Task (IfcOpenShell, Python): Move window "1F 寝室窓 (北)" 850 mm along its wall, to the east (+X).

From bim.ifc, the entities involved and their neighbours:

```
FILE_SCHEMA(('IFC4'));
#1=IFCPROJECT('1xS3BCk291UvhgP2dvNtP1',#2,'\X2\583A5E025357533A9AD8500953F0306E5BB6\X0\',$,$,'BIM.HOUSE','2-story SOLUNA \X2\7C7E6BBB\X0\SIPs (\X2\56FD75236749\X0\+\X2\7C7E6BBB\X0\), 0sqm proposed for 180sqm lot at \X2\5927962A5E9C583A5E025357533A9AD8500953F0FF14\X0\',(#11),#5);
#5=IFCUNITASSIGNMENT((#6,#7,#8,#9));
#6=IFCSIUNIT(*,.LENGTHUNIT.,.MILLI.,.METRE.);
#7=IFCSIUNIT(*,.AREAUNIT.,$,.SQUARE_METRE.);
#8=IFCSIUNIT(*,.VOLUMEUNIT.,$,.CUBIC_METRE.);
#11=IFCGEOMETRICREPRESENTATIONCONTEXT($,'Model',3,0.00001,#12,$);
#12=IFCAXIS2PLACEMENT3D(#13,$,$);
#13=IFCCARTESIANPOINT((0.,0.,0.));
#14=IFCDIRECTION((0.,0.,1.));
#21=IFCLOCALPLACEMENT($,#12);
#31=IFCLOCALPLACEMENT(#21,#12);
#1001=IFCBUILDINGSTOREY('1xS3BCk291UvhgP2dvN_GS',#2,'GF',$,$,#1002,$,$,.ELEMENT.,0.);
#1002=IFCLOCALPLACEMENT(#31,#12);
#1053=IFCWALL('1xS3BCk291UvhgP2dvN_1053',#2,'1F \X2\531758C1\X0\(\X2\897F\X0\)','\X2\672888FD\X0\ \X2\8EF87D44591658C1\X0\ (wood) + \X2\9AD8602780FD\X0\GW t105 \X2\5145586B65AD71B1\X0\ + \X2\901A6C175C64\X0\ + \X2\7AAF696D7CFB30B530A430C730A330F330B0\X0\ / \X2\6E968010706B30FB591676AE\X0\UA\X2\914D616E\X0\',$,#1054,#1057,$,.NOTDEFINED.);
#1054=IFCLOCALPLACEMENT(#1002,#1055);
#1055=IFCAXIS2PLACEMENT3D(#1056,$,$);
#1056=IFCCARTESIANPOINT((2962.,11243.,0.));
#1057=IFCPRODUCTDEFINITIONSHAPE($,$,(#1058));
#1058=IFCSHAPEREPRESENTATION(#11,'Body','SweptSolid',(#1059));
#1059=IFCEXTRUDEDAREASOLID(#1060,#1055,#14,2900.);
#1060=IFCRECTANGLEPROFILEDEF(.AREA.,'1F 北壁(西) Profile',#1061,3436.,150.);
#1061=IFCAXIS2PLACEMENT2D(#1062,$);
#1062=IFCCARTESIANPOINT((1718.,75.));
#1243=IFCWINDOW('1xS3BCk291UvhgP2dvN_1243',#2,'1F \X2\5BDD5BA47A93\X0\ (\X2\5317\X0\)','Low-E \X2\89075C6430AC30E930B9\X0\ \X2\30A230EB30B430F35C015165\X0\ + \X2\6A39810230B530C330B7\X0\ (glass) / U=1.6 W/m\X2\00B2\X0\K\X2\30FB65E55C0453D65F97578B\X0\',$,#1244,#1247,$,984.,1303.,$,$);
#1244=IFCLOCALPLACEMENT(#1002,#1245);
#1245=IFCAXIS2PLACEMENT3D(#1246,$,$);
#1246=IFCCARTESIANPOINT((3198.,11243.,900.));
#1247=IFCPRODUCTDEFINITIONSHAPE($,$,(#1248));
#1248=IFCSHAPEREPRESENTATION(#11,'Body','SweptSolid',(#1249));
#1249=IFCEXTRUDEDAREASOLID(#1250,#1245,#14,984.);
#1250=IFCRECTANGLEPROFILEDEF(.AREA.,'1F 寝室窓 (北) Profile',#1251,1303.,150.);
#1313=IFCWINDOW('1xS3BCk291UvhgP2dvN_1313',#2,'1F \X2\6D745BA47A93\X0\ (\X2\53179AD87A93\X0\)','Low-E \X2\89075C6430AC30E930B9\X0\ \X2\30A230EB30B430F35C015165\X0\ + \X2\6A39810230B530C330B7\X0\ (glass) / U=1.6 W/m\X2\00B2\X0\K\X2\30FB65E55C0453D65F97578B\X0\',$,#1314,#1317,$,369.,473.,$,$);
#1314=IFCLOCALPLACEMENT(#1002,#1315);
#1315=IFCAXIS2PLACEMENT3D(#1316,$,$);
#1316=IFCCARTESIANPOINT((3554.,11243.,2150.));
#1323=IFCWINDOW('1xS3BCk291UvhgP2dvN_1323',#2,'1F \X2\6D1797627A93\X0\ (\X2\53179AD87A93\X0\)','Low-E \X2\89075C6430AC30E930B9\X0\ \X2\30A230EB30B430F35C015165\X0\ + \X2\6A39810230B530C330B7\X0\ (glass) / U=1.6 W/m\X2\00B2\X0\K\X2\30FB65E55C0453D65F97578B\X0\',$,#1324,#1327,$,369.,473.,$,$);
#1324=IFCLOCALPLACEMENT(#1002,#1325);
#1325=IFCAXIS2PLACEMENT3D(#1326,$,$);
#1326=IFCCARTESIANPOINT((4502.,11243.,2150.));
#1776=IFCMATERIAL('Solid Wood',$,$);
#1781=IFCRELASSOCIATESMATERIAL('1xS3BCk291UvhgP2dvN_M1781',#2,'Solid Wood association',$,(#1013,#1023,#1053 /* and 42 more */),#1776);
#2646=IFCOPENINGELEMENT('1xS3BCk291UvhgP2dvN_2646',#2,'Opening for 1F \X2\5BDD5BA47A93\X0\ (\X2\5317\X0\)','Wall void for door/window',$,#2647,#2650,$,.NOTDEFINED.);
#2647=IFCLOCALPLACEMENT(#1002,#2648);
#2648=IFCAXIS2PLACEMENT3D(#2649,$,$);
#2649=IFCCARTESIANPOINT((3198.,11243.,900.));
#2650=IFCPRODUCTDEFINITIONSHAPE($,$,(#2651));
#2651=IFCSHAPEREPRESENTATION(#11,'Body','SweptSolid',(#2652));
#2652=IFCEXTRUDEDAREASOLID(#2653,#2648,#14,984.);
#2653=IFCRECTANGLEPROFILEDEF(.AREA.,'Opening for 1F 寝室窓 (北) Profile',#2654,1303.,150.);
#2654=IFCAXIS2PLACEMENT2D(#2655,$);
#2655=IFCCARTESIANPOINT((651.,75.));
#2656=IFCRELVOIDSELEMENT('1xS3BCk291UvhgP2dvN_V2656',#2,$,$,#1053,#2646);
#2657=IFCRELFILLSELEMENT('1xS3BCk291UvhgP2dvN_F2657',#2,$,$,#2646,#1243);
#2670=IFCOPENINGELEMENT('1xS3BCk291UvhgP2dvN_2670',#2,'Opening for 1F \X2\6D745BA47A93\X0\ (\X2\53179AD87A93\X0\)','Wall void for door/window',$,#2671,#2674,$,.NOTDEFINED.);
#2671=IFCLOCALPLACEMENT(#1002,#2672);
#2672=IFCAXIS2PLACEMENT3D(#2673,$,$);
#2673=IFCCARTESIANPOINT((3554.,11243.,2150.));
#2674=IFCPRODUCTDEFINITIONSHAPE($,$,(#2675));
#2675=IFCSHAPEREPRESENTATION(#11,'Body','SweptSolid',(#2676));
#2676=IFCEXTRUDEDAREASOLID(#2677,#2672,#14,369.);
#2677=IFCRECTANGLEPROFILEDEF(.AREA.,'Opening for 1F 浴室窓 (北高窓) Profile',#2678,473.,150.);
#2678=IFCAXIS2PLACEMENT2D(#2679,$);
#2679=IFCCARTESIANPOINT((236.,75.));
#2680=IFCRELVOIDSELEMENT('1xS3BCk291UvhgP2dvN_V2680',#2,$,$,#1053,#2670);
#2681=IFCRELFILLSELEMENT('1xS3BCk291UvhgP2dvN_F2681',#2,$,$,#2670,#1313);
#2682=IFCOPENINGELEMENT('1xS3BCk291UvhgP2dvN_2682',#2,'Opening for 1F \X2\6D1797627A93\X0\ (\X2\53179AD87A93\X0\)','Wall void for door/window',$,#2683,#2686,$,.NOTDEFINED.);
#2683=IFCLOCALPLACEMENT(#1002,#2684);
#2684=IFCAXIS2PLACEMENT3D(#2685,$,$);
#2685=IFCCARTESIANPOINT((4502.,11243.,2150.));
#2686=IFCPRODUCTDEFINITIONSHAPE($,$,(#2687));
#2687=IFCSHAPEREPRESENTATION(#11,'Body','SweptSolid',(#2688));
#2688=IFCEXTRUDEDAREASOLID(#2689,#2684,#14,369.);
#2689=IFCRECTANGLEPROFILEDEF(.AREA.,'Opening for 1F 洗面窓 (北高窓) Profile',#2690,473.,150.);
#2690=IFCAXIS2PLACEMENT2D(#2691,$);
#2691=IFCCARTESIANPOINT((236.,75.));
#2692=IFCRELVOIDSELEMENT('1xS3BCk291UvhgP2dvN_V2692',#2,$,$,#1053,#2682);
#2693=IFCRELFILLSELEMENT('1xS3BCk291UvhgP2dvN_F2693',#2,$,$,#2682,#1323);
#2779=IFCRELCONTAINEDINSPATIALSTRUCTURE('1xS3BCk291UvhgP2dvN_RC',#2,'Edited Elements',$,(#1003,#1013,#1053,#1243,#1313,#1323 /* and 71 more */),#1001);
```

```python
import ifcopenshell
import ifcopenshell.api.geometry
import ifcopenshell.util.placement
import ifcopenshell.util.unit

model = ifcopenshell.open("bim.ifc")
unit_scale = ifcopenshell.util.unit.calculate_unit_scale(model)

window = model.by_guid("1xS3BCk291UvhgP2dvN_1243")
opening = window.FillsVoids[0].RelatingOpeningElement
wall = opening.VoidsElements[0].RelatingBuildingElement

wall_matrix = ifcopenshell.util.placement.get_local_placement(wall.ObjectPlacement)
shift = wall_matrix[:3, 0] * 0.85 / unit_scale
before = ifcopenshell.util.placement.get_local_placement(window.ObjectPlacement)[:3, 3].copy()

# The window is not placed relative to its opening, so move both.
for product in (opening, window):
    matrix = ifcopenshell.util.placement.get_local_placement(product.ObjectPlacement)
    matrix[:3, 3] += shift
    ifcopenshell.api.geometry.edit_object_placement(model, product=product, matrix=matrix, is_si=False)

after = ifcopenshell.util.placement.get_local_placement(window.ObjectPlacement)[:3, 3]
print("window moved by", (after - before).round(3) + 0.0)

model.write("bim_v2.ifc")
```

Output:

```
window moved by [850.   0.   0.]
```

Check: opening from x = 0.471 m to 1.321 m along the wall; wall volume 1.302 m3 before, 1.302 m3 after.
